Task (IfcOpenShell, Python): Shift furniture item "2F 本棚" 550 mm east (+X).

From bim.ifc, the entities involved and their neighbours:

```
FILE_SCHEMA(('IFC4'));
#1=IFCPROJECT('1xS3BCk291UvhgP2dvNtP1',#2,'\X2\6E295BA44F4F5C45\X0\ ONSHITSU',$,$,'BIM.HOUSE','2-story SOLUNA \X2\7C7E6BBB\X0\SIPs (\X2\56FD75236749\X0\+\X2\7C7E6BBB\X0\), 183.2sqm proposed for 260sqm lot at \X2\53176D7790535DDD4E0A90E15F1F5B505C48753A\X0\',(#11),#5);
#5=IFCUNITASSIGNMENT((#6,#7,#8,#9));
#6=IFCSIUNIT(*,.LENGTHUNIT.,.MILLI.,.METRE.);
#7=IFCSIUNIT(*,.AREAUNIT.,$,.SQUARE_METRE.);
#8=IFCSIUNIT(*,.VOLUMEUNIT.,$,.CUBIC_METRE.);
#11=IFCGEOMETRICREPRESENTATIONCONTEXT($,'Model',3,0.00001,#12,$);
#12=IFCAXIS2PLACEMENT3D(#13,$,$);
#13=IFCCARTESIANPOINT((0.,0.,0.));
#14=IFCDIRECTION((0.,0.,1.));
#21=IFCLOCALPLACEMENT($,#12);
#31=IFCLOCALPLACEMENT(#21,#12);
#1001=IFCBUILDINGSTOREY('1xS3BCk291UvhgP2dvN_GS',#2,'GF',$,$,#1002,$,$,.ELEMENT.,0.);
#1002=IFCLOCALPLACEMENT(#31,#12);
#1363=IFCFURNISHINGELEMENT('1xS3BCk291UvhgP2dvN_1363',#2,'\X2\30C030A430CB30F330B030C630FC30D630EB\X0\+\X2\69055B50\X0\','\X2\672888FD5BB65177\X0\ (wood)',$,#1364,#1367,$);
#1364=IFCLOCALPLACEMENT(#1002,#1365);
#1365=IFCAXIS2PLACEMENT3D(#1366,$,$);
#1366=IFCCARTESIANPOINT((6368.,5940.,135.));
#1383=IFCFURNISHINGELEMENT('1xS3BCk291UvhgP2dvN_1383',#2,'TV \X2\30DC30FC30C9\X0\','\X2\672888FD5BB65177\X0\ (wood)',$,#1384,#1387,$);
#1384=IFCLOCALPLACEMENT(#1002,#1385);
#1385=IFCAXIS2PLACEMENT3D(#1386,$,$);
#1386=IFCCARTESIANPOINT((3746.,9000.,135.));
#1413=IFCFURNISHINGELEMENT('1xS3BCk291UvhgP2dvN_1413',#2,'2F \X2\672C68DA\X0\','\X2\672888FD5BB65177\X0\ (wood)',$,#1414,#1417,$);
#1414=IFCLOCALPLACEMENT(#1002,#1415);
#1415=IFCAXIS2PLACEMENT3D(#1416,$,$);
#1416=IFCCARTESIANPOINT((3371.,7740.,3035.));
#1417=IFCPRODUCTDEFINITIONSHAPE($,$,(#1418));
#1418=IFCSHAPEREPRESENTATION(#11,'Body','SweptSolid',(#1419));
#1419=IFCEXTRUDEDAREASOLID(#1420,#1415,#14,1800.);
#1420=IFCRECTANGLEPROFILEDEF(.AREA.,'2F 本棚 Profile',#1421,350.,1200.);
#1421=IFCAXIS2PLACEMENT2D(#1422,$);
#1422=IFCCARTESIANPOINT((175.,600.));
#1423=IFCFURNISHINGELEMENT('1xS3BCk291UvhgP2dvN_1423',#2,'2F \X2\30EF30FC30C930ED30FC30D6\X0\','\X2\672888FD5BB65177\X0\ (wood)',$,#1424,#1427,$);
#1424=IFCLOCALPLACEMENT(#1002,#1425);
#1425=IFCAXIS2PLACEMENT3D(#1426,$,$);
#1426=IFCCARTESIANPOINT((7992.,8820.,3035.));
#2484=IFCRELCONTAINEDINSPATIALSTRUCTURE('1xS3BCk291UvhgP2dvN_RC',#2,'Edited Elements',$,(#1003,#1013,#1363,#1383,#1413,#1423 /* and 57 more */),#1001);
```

```python
import ifcopenshell
import ifcopenshell.api.geometry
import ifcopenshell.util.placement
import ifcopenshell.util.unit

model = ifcopenshell.open("bim.ifc")
unit_scale = ifcopenshell.util.unit.calculate_unit_scale(model)

item = model.by_id(1413)
matrix = ifcopenshell.util.placement.get_local_placement(item.ObjectPlacement)
matrix[0, 3] += 0.55 / unit_scale
ifcopenshell.api.geometry.edit_object_placement(model, product=item, matrix=matrix, is_si=False)

print(ifcopenshell.util.placement.get_local_placement(item.ObjectPlacement).round(3) + 0.0)

model.write("bim-out.ifc")
```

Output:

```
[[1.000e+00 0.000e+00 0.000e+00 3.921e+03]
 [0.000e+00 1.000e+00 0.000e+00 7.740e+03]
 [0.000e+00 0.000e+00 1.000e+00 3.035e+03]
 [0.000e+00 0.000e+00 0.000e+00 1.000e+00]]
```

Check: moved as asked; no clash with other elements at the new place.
